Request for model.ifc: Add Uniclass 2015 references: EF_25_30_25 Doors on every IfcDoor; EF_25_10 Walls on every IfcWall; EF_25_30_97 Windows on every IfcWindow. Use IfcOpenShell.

First a look at what the model holds.

```python
import ifcopenshell

model = ifcopenshell.open("model.ifc")
print(model.schema)
print("classifications:", [c.Name for c in model.by_type("IfcClassification")])
for ifc_class in ("IfcDoor", "IfcRoof", "IfcStair", "IfcWall", "IfcWindow"):
    print(ifc_class, len(model.by_type(ifc_class)))
```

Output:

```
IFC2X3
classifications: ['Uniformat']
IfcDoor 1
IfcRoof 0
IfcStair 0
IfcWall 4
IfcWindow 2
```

```python
import ifcopenshell
import ifcopenshell.api.classification

model = ifcopenshell.open("model.ifc")

# IFC2X3 requires Source and Edition and has no link from the project to the system.
system = model.create_entity("IfcClassification", Source="NBS", Edition="2015", Name="Uniclass 2015")

codes = {
    "IfcDoor": ("EF_25_30_25", "Doors"),
    "IfcWall": ("EF_25_10", "Walls"),
    "IfcWindow": ("EF_25_30_97", "Windows"),
}
for ifc_class, (code, name) in codes.items():
    products = model.by_type(ifc_class)
    ifcopenshell.api.classification.add_reference(
        model, products=products, classification=system, identification=code, name=name
    )
    print(code, len(products))

model.write("model-out.ifc")
```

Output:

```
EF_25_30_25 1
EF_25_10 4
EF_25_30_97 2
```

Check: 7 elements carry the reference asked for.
